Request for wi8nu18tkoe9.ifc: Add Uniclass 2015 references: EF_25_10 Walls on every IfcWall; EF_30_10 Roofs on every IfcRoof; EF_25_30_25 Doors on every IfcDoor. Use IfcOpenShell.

First a look at what the model holds.

```python
import ifcopenshell

model = ifcopenshell.open("wi8nu18tkoe9.ifc")
print(model.schema)
print("classifications:", [c.Name for c in model.by_type("IfcClassification")])
for ifc_class in ("IfcDoor", "IfcRoof", "IfcStair", "IfcWall", "IfcWindow"):
    print(ifc_class, len(model.by_type(ifc_class)))
```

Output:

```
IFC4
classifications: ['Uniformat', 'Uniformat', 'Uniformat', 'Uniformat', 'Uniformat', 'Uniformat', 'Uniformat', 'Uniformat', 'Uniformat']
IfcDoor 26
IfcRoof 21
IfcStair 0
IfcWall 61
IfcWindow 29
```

```python
import ifcopenshell
import ifcopenshell.api.classification

model = ifcopenshell.open("wi8nu18tkoe9.ifc")

system = ifcopenshell.api.classification.add_classification(model, classification="Uniclass 2015")

codes = {
    "IfcWall": ("EF_25_10", "Walls"),
    "IfcRoof": ("EF_30_10", "Roofs"),
    "IfcDoor": ("EF_25_30_25", "Doors"),
}
for ifc_class, (code, name) in codes.items():
    products = model.by_type(ifc_class)
    ifcopenshell.api.classification.add_reference(
        model, products=products, classification=system, identification=code, name=name
    )
    print(code, len(products))

model.write("wi8nu18tkoe9-out.ifc")
```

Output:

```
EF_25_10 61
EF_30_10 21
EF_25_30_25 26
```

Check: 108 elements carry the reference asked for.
